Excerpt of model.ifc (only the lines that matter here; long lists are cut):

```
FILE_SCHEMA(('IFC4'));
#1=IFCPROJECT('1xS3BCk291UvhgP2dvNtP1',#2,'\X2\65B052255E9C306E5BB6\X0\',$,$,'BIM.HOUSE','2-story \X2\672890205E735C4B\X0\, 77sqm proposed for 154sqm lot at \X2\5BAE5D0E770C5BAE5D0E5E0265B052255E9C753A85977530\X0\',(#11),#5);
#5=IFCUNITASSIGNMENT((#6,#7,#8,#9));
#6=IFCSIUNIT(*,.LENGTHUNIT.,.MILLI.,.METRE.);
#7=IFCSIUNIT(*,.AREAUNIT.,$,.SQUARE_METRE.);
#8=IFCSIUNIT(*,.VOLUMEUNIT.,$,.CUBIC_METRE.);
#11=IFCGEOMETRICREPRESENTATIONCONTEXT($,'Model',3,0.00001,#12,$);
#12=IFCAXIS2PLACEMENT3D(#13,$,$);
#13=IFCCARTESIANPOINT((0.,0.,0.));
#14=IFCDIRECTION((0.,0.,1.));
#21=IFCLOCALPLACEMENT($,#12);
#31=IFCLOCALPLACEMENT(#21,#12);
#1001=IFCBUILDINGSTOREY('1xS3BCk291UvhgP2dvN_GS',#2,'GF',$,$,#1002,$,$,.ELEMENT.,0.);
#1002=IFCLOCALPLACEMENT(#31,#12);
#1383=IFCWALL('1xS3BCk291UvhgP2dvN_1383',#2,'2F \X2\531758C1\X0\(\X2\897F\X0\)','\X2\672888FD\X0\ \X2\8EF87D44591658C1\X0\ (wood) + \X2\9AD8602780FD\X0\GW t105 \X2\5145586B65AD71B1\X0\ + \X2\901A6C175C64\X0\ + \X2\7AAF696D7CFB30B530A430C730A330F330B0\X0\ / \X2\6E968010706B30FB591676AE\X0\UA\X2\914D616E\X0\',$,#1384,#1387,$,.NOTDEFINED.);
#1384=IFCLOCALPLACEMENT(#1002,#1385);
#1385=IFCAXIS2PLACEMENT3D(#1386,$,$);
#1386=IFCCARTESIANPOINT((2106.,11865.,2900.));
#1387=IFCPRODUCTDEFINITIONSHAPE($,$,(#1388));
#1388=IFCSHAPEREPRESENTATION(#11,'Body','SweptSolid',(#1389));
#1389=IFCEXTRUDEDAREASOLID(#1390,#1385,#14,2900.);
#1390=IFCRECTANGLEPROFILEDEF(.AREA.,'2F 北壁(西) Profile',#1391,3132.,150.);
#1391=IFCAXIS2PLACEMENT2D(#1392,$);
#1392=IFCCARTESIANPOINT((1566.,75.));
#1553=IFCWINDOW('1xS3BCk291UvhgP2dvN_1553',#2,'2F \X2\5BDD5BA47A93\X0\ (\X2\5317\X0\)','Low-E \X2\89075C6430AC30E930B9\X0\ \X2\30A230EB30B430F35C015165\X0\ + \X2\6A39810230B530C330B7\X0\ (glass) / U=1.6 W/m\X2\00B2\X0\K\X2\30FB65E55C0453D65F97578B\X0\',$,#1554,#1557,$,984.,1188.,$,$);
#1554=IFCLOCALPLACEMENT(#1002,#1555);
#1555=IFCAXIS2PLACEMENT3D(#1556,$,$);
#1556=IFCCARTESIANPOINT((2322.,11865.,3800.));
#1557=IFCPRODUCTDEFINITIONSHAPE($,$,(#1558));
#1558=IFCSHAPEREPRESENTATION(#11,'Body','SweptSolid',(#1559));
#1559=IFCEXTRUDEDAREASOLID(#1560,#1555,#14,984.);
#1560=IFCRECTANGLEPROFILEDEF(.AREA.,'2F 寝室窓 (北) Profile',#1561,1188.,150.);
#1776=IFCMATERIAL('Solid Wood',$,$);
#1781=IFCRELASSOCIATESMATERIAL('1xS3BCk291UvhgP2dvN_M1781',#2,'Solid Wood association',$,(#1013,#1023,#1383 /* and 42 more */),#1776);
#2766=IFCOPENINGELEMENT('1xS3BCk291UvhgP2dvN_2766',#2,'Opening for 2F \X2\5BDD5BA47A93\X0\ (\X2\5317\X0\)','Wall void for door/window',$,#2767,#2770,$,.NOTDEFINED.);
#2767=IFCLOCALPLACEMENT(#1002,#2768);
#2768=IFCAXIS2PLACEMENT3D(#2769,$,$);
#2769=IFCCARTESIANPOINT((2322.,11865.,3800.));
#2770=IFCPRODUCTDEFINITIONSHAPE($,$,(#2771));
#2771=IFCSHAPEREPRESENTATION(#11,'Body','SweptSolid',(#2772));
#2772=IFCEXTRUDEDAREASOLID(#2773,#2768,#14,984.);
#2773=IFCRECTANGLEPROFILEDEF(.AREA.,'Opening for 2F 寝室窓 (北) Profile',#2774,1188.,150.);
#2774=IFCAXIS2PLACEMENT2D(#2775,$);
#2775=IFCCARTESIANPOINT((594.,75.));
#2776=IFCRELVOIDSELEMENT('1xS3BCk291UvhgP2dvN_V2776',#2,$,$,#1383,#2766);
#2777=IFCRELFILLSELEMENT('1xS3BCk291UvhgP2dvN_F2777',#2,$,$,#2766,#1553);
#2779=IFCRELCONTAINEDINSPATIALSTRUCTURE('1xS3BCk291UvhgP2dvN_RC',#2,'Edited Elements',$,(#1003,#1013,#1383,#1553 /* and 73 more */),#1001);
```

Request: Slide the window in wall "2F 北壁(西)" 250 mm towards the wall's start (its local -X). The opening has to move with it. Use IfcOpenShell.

```python
import ifcopenshell
import ifcopenshell.api.geometry
import ifcopenshell.util.placement
import ifcopenshell.util.unit

model = ifcopenshell.open("model.ifc")
unit_scale = ifcopenshell.util.unit.calculate_unit_scale(model)

window = model.by_guid("1xS3BCk291UvhgP2dvN_1553")
opening = window.FillsVoids[0].RelatingOpeningElement
wall = opening.VoidsElements[0].RelatingBuildingElement

wall_matrix = ifcopenshell.util.placement.get_local_placement(wall.ObjectPlacement)
shift = wall_matrix[:3, 0] * -0.25 / unit_scale
before = ifcopenshell.util.placement.get_local_placement(window.ObjectPlacement)[:3, 3].copy()

# The window is not placed relative to its opening, so move both.
for product in (opening, window):
    matrix = ifcopenshell.util.placement.get_local_placement(product.ObjectPlacement)
    matrix[:3, 3] += shift
    ifcopenshell.api.geometry.edit_object_placement(model, product=product, matrix=matrix, is_si=False)

after = ifcopenshell.util.placement.get_local_placement(window.ObjectPlacement)[:3, 3]
print("window moved by", (after - before).round(3) + 0.0)

model.write("model_rev.ifc")
```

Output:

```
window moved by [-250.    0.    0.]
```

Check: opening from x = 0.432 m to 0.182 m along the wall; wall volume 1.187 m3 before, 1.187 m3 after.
